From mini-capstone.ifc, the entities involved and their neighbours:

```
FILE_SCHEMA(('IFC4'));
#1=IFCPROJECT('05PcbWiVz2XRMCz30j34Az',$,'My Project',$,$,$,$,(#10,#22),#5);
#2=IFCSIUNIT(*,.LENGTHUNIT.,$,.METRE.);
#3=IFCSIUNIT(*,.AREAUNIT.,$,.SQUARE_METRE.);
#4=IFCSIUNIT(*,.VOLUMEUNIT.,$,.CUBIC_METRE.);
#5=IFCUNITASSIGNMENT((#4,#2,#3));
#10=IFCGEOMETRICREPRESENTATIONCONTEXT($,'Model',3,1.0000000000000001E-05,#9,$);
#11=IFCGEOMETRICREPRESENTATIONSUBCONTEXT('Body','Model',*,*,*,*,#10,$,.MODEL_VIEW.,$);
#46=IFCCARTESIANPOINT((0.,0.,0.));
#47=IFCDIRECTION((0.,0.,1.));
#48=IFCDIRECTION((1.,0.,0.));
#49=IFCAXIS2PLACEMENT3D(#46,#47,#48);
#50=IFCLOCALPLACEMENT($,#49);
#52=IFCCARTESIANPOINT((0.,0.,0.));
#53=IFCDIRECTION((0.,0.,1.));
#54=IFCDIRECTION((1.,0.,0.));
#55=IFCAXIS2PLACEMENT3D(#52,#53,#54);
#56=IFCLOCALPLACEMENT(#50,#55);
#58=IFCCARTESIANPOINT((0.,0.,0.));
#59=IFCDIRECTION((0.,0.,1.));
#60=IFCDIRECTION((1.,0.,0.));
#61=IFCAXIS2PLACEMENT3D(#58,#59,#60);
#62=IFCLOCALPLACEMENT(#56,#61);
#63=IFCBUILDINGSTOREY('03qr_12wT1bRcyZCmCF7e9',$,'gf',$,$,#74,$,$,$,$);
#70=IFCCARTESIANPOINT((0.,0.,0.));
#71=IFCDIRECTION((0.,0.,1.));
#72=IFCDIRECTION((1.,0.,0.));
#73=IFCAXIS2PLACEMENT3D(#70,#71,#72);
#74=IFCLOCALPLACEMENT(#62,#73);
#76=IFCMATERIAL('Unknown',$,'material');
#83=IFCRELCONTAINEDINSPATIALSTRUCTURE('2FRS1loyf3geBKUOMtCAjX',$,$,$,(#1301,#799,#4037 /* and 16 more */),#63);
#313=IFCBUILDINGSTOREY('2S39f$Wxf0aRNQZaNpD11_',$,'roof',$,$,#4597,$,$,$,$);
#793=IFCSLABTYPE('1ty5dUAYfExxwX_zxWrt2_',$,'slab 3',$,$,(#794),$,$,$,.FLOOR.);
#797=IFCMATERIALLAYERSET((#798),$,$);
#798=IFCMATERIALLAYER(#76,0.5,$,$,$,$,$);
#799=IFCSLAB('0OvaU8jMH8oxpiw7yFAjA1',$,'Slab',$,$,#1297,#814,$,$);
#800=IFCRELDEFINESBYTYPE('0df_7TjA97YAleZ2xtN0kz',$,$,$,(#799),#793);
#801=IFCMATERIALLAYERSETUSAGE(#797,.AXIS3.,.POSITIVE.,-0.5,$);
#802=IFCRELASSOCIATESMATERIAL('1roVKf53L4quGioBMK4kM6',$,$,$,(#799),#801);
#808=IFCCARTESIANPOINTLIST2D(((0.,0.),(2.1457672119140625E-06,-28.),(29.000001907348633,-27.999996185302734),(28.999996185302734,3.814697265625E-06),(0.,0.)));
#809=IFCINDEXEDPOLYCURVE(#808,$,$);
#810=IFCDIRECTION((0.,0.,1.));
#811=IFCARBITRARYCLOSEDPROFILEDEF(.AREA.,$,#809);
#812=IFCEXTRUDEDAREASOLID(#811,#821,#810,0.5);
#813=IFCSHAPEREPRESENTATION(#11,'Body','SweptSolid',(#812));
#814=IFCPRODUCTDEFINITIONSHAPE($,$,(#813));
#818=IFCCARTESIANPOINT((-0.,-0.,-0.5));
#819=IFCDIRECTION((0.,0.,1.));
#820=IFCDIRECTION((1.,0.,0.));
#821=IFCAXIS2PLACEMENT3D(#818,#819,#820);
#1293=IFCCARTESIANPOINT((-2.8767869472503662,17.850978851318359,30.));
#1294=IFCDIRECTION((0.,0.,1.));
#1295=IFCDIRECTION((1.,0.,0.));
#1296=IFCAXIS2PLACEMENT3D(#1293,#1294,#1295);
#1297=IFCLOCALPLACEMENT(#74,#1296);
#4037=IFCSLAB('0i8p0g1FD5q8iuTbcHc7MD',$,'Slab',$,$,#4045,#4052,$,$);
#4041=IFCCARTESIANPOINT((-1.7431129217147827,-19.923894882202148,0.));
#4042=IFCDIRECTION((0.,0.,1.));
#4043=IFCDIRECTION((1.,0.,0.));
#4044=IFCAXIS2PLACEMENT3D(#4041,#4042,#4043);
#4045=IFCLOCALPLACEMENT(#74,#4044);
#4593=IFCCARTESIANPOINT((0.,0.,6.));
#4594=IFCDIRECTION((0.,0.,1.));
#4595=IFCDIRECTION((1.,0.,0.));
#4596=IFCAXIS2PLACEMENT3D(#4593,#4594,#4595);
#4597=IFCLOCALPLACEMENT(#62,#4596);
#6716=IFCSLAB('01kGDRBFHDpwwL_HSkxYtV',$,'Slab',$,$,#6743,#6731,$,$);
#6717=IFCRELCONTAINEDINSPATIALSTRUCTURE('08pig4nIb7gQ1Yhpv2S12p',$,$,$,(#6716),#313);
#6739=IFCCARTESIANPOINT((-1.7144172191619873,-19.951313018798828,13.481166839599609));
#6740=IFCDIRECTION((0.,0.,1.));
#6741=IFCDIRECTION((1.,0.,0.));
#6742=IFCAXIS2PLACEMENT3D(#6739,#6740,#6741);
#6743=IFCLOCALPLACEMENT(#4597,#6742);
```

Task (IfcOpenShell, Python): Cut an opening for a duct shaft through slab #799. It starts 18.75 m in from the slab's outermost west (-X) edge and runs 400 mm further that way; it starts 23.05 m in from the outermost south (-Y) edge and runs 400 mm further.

```python
import numpy as np
import ifcopenshell
import ifcopenshell.api.feature
import ifcopenshell.api.geometry
import ifcopenshell.api.root
import ifcopenshell.geom
import ifcopenshell.util.placement
import ifcopenshell.util.representation
import ifcopenshell.util.shape
import ifcopenshell.util.unit

model = ifcopenshell.open("mini-capstone.ifc")
unit_scale = ifcopenshell.util.unit.calculate_unit_scale(model)
settings = ifcopenshell.geom.settings()


def volume(element):
    """Net volume in cubic metres, openings subtracted."""
    shape = ifcopenshell.geom.create_shape(settings, element)
    return ifcopenshell.util.shape.get_volume(shape.geometry)


slab = model.by_guid("0OvaU8jMH8oxpiw7yFAjA1")
before = volume(slab)

# Extent in the slab's own axes, in metres. The edges named are its -X and -Y sides.
slab_shape = ifcopenshell.geom.create_shape(settings, slab)
vertices = ifcopenshell.util.shape.get_vertices(slab_shape.geometry)
x_min, y_min, bottom = vertices.min(axis=0)
top = vertices[:, 2].max()

opening = ifcopenshell.api.root.create_entity(model, ifc_class="IfcOpeningElement", name="Duct shaft opening", predefined_type="OPENING")
context = ifcopenshell.util.representation.get_context(model, "Model", "Body", "MODEL_VIEW")
width, depth = 0.4, 0.4
outline = [(0.0, 0.0), (width, 0.0), (width, depth), (0.0, depth), (0.0, 0.0)]
# Overshoot both faces by 50 mm so the cut is clean.
shape = ifcopenshell.api.geometry.add_slab_representation(
    model, context=context, depth=top - bottom + 0.1, polyline=outline
)
ifcopenshell.api.geometry.assign_representation(model, product=opening, representation=shape)

matrix = ifcopenshell.util.placement.get_local_placement(slab.ObjectPlacement)
matrix[:, 3] = matrix @ np.append(np.array([x_min + 18.75, y_min + 23.05, bottom - 0.05]) / unit_scale, 1.0)
ifcopenshell.api.geometry.edit_object_placement(model, product=opening, matrix=matrix, is_si=False)
ifcopenshell.api.feature.add_feature(model, feature=opening, element=slab)

after = volume(slab)

print(f"slab volume {before:.3f} -> {after:.3f} m3")

model.write("mini-capstone_edited.ifc")
```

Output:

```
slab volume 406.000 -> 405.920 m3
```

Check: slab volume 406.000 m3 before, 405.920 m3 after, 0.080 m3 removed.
